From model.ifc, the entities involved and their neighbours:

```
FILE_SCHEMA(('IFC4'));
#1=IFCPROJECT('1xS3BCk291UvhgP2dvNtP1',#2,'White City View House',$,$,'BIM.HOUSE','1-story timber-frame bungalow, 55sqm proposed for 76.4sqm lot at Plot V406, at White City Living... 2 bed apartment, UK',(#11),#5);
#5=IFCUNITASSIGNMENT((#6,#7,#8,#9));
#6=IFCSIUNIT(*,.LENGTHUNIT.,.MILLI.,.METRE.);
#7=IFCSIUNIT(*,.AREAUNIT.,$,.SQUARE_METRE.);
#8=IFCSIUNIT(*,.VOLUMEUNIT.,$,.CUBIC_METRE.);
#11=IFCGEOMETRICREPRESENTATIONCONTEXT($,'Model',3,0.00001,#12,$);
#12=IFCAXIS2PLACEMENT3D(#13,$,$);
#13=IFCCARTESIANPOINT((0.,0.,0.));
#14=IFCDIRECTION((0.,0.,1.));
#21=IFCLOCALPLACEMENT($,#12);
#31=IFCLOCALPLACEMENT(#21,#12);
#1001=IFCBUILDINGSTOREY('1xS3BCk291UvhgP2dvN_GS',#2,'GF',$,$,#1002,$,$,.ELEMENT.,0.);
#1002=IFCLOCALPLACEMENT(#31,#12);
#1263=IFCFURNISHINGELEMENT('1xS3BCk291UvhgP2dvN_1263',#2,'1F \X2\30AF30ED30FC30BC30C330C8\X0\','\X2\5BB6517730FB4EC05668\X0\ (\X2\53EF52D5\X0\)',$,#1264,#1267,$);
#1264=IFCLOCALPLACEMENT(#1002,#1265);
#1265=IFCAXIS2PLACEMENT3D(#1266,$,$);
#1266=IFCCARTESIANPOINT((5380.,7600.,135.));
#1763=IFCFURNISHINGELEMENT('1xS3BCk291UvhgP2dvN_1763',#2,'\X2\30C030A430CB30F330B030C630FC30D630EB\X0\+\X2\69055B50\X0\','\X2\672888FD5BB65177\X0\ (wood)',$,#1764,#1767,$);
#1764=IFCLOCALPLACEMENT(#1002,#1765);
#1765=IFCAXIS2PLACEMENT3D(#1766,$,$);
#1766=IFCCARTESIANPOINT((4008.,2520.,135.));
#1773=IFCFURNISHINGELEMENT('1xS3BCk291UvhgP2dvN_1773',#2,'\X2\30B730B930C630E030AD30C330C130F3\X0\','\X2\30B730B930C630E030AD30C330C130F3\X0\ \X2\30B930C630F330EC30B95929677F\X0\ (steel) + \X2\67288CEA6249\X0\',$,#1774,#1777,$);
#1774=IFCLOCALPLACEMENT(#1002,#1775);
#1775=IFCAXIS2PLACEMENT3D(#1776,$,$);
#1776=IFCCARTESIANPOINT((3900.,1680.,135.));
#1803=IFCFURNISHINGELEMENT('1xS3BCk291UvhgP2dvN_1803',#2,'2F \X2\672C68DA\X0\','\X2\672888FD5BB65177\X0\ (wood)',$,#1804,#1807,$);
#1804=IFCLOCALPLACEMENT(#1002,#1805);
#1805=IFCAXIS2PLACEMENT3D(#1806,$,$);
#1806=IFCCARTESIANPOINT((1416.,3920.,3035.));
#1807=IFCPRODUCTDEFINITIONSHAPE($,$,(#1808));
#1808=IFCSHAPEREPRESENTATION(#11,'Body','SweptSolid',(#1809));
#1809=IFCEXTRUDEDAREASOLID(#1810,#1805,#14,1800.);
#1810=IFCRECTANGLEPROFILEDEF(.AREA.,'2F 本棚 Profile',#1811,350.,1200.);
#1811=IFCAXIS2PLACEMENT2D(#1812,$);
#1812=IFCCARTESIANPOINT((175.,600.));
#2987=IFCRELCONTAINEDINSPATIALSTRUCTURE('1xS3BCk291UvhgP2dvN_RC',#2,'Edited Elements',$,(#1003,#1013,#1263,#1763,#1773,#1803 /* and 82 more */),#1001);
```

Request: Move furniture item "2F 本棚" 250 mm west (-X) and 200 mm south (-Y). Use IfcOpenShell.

```python
import ifcopenshell
import ifcopenshell.api.geometry
import ifcopenshell.util.placement
import ifcopenshell.util.unit

model = ifcopenshell.open("model.ifc")
unit_scale = ifcopenshell.util.unit.calculate_unit_scale(model)

item = model.by_id(1803)
matrix = ifcopenshell.util.placement.get_local_placement(item.ObjectPlacement)
matrix[0, 3] -= 0.25 / unit_scale
matrix[1, 3] -= 0.2 / unit_scale
ifcopenshell.api.geometry.edit_object_placement(model, product=item, matrix=matrix, is_si=False)

print(ifcopenshell.util.placement.get_local_placement(item.ObjectPlacement).round(3) + 0.0)

model.write("model_updated.ifc")
```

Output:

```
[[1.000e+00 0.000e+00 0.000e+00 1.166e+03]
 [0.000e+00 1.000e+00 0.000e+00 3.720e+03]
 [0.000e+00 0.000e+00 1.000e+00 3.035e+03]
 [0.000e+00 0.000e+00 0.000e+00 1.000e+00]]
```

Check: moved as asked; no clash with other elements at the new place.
